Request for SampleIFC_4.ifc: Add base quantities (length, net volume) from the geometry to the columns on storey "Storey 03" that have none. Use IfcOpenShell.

First a look at what the model holds.

```python
import ifcopenshell
import ifcopenshell.util.element
import ifcopenshell.util.unit

model = ifcopenshell.open("SampleIFC_4.ifc")
print(model.schema)
for unit_type in ("LENGTHUNIT", "AREAUNIT", "VOLUMEUNIT"):
    print(unit_type, ifcopenshell.util.unit.calculate_unit_scale(model, unit_type))
storey = next(s for s in model.by_type("IfcBuildingStorey") if s.Name == "Storey 03")
columns = [e for e in ifcopenshell.util.element.get_decomposition(storey) if e.is_a("IfcColumn")]
for e in sorted(columns, key=lambda e: e.id()):
    print(e.id(), e.is_a(), e.Name, list(ifcopenshell.util.element.get_psets(e, qtos_only=True)), sep=" | ")
```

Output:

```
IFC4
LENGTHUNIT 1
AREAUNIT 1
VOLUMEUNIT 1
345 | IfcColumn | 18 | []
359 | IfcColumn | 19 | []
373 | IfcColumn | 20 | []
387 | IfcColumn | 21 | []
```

```python
import ifcopenshell
import ifcopenshell.api.pset
import ifcopenshell.geom
import ifcopenshell.util.element
import ifcopenshell.util.shape
import ifcopenshell.util.unit

model = ifcopenshell.open("SampleIFC_4.ifc")
unit_scale = ifcopenshell.util.unit.calculate_unit_scale(model)
volume_scale = ifcopenshell.util.unit.calculate_unit_scale(model, "VOLUMEUNIT")
settings = ifcopenshell.geom.settings()

storey = next(s for s in model.by_type("IfcBuildingStorey") if s.Name == "Storey 03")
columns = [e for e in ifcopenshell.util.element.get_decomposition(storey) if e.is_a("IfcColumn")]

for e in sorted(columns, key=lambda e: e.id()):
    if ifcopenshell.util.element.get_psets(e, qtos_only=True, should_inherit=False):
        continue
    # Geometry comes back in metres, in the element's own axes.
    shape = ifcopenshell.geom.create_shape(settings, e)
    values = {
        "Length": ifcopenshell.util.shape.get_z(shape.geometry) / unit_scale,
        "NetVolume": ifcopenshell.util.shape.get_volume(shape.geometry) / volume_scale,
    }
    qto = ifcopenshell.api.pset.add_qto(model, product=e, name="Qto_ColumnBaseQuantities")
    ifcopenshell.api.pset.edit_qto(model, qto=qto, properties=values)
    print(e.id(), {k: round(v, 3) for k, v in values.items()})

model.write("SampleIFC_4-out.ifc")
```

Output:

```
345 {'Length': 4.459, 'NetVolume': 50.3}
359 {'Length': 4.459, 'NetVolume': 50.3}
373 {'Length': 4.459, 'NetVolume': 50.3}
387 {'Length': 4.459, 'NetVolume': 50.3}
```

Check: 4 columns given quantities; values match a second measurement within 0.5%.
